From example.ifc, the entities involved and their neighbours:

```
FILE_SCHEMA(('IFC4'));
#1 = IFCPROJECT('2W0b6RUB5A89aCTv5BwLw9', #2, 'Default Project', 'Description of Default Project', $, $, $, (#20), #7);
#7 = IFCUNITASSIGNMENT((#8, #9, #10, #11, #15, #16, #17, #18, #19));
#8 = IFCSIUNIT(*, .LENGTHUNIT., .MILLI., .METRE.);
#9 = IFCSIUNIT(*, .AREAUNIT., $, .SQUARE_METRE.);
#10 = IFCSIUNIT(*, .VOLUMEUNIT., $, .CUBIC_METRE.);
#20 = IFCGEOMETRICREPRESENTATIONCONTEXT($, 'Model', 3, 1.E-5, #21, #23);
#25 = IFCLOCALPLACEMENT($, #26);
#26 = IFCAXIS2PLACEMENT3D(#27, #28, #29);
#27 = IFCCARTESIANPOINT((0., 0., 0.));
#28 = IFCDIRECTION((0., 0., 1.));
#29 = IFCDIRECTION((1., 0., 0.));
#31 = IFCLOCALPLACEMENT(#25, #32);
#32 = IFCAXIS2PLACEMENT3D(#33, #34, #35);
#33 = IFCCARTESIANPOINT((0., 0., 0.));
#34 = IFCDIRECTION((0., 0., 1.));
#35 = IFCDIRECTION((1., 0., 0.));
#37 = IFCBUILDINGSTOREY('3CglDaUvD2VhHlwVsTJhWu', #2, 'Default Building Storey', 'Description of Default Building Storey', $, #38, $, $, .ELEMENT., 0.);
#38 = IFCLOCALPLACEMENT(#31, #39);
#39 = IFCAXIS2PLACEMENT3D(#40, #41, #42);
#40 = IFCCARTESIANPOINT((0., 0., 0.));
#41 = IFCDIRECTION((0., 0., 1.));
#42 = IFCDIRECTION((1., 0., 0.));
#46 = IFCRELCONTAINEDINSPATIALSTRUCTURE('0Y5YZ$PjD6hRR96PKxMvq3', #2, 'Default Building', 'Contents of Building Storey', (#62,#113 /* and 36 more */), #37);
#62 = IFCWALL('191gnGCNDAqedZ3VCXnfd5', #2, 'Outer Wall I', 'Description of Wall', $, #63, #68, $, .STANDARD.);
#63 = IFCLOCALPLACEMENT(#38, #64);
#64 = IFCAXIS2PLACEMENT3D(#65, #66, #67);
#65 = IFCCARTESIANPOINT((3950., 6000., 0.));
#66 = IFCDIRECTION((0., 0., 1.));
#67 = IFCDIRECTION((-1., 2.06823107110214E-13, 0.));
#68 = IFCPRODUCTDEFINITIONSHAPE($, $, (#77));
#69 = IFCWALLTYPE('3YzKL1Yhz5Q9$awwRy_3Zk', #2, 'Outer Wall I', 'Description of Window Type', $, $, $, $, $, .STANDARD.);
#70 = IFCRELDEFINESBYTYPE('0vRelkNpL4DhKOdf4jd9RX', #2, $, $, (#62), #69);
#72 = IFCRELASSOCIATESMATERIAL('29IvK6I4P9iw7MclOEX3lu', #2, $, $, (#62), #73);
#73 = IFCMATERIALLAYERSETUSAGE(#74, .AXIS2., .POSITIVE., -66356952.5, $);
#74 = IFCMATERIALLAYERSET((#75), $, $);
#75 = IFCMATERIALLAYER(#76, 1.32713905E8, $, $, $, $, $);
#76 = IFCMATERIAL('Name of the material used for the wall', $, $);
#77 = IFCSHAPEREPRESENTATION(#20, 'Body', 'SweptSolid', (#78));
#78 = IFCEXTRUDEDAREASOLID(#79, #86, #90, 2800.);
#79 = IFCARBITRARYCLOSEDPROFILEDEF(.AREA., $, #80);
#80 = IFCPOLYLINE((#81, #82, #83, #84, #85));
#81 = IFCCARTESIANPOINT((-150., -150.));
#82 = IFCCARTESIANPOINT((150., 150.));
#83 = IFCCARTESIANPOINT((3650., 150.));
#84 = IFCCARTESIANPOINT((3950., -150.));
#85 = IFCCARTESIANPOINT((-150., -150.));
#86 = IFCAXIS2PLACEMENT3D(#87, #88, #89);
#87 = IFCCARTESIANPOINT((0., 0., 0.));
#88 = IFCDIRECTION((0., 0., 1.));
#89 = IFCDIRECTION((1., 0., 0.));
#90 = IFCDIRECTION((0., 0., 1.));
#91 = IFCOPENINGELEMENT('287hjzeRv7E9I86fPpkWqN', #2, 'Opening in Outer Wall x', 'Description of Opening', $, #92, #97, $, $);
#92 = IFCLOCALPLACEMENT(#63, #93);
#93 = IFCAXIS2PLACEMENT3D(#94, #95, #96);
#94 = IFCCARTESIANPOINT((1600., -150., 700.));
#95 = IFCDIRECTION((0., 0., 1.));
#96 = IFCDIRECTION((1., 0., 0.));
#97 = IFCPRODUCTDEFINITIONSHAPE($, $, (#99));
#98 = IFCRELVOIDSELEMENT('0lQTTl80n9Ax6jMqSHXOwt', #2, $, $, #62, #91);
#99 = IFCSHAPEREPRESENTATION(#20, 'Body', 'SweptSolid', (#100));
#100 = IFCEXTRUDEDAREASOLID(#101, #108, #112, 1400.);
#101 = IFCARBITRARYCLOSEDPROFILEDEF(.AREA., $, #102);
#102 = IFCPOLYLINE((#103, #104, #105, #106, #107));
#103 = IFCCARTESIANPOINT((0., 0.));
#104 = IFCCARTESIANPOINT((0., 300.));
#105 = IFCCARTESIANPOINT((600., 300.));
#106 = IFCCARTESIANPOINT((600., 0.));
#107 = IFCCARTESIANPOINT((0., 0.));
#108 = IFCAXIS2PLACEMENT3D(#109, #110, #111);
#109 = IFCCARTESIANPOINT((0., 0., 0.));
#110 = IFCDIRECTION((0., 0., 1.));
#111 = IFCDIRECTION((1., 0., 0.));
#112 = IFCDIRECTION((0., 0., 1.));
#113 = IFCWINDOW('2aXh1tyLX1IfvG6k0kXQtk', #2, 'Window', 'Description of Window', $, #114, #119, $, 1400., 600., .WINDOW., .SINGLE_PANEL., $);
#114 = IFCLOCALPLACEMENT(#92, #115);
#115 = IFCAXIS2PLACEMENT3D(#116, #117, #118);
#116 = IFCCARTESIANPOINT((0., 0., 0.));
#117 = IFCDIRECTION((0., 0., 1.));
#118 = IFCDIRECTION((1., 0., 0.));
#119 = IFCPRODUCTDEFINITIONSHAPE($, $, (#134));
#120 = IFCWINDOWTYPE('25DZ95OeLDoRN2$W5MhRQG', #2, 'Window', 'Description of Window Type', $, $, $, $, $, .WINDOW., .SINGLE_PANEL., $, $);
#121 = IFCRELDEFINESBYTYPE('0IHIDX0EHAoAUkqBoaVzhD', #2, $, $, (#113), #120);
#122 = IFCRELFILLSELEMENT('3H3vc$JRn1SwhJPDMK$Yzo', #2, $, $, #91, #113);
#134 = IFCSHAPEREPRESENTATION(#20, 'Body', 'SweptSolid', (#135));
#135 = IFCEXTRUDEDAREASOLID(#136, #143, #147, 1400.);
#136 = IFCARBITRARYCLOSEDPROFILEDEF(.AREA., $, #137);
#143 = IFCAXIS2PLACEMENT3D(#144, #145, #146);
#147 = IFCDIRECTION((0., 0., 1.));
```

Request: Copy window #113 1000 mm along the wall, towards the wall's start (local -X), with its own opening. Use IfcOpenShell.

```python
import ifcopenshell
import ifcopenshell.api.feature
import ifcopenshell.api.geometry
import ifcopenshell.api.root
import ifcopenshell.geom
import ifcopenshell.util.element
import ifcopenshell.util.placement
import ifcopenshell.util.shape
import ifcopenshell.util.unit

model = ifcopenshell.open("example.ifc")
unit_scale = ifcopenshell.util.unit.calculate_unit_scale(model)
settings = ifcopenshell.geom.settings()


def volume(element):
    """Net volume in cubic metres, openings subtracted."""
    shape = ifcopenshell.geom.create_shape(settings, element)
    return ifcopenshell.util.shape.get_volume(shape.geometry)


def reuse_history(source, copy):
    """copy_class also copies each property set's owner history, people and application; keep the originals."""
    for rel in copy.IsDefinedBy:
        if rel.is_a("IfcRelDefinesByProperties") and (history := rel.RelatingPropertyDefinition.OwnerHistory):
            rel.RelatingPropertyDefinition.OwnerHistory = source.OwnerHistory
            ifcopenshell.util.element.remove_deep2(model, history)


window = model.by_id(113)
opening = window.FillsVoids[0].RelatingOpeningElement
wall = opening.VoidsElements[0].RelatingBuildingElement
before = volume(wall)
shift = ifcopenshell.util.placement.get_local_placement(wall.ObjectPlacement)[:3, 0] * -1 / unit_scale

# copy_class copies the void relationship, type, container and properties, but no geometry.
new_opening = ifcopenshell.api.root.copy_class(model, product=opening)
new_opening.Representation = ifcopenshell.util.element.copy_deep(
    model, opening.Representation, exclude=["IfcGeometricRepresentationContext", "IfcRepresentationMap"]
)
new_window = ifcopenshell.api.root.copy_class(model, product=window)
new_window.Representation = ifcopenshell.util.element.copy_deep(
    model, window.Representation, exclude=["IfcGeometricRepresentationContext", "IfcRepresentationMap"]
)
reuse_history(window, new_window)
ifcopenshell.api.feature.add_filling(model, opening=new_opening, element=new_window)

for old, new in ((opening, new_opening), (window, new_window)):
    matrix = ifcopenshell.util.placement.get_local_placement(old.ObjectPlacement)
    matrix[:3, 3] += shift
    ifcopenshell.api.geometry.edit_object_placement(model, product=new, matrix=matrix, is_si=False)

after = volume(wall)

print(f"wall volume {before:.3f} -> {after:.3f} m3")

model.write("example-out.ifc")
```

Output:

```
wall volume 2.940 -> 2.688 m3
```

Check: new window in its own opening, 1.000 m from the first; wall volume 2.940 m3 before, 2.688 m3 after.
